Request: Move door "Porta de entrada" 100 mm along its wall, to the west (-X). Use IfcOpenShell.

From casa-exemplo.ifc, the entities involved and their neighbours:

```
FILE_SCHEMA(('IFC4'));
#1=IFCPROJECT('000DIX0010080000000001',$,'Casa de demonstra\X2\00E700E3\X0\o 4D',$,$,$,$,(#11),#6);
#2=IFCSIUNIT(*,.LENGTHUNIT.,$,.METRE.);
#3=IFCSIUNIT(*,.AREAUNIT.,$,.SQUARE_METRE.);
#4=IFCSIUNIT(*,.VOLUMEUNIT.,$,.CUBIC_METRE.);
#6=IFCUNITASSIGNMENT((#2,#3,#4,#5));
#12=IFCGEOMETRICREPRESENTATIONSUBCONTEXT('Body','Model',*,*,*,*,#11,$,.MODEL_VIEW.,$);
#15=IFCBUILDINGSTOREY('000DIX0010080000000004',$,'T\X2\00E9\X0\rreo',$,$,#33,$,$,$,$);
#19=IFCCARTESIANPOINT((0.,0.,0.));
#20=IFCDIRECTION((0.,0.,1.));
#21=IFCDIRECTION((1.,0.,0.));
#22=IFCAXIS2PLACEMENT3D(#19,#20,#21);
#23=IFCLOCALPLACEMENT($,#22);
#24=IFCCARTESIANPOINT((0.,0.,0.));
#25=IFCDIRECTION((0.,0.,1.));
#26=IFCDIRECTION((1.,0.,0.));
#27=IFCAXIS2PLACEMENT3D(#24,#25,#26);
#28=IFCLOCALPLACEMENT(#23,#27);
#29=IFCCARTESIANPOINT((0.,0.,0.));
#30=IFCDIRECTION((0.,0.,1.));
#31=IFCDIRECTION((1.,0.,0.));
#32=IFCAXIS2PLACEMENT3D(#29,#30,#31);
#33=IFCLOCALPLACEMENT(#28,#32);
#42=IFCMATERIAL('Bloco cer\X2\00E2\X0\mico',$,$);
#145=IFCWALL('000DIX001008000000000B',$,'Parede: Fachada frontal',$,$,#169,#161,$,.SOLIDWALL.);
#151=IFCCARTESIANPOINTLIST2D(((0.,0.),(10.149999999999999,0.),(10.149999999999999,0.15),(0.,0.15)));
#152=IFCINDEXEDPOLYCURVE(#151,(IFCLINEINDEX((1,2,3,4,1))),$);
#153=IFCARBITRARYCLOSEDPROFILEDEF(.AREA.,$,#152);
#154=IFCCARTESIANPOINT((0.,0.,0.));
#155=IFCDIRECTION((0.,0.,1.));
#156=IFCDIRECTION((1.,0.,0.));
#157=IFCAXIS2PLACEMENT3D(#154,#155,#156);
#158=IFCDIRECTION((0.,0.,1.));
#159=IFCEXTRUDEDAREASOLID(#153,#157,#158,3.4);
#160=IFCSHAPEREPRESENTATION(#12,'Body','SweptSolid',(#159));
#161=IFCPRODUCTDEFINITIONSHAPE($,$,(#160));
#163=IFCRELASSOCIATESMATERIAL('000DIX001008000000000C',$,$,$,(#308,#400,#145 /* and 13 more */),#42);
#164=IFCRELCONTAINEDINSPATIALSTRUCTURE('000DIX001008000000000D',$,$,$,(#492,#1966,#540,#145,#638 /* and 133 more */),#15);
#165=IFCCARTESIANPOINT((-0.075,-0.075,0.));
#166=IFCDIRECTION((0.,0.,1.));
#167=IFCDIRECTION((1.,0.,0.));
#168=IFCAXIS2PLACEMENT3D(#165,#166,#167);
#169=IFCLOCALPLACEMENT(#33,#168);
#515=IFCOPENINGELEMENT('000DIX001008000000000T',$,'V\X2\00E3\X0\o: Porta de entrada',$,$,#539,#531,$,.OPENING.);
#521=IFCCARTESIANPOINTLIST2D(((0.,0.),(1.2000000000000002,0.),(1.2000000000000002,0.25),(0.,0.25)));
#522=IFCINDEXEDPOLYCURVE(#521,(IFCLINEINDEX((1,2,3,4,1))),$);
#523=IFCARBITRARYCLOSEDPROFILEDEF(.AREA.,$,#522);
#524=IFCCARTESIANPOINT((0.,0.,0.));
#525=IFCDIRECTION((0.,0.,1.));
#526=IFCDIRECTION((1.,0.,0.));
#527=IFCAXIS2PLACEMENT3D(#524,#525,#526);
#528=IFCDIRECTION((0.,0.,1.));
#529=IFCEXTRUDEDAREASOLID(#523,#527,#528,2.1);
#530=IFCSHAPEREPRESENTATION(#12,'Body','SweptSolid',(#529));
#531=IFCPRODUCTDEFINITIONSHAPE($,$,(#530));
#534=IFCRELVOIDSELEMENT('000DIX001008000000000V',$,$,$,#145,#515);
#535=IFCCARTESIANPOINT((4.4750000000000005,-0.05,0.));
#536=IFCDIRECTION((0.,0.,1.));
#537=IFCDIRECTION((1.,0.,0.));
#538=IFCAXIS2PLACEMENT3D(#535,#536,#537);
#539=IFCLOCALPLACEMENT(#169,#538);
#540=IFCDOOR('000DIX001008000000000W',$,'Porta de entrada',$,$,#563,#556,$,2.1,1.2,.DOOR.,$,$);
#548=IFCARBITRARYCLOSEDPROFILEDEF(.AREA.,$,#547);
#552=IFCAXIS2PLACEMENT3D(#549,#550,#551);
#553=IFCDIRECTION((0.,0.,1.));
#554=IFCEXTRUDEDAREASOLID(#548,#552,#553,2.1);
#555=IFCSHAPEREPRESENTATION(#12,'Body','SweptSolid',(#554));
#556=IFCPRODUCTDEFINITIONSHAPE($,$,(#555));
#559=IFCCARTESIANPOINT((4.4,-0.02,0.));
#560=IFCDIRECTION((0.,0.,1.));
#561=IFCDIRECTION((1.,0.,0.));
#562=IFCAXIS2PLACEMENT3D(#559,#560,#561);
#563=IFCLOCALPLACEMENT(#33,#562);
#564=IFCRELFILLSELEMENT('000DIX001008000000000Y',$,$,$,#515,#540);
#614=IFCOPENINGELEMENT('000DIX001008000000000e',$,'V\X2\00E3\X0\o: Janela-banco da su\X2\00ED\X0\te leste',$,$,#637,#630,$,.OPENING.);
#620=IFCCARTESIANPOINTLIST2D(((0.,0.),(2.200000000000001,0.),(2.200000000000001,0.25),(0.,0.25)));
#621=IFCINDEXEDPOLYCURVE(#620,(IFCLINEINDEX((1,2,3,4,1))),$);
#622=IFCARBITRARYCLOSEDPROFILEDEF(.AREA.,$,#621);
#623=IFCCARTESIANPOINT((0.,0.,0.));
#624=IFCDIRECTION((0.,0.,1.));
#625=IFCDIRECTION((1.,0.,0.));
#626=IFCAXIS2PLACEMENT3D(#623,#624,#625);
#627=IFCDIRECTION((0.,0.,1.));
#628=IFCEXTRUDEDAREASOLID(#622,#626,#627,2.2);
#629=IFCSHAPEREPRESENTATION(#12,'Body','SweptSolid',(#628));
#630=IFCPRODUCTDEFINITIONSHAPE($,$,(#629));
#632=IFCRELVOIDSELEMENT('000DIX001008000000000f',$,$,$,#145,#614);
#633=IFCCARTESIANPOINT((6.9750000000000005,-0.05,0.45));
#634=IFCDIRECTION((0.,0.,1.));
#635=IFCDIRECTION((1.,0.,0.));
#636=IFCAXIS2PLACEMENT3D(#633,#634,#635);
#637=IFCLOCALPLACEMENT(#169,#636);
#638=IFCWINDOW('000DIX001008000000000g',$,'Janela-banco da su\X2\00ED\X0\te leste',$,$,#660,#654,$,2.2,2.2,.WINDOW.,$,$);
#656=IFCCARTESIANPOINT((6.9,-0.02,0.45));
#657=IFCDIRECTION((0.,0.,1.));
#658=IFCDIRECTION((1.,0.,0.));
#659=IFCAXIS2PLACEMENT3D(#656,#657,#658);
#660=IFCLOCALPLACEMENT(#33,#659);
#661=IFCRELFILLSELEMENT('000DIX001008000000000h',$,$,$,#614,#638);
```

```python
import ifcopenshell
import ifcopenshell.api.geometry
import ifcopenshell.util.placement

model = ifcopenshell.open("casa-exemplo.ifc")

door = model.by_id(540)
opening = door.FillsVoids[0].RelatingOpeningElement
wall = opening.VoidsElements[0].RelatingBuildingElement

wall_matrix = ifcopenshell.util.placement.get_local_placement(wall.ObjectPlacement)
shift = wall_matrix[:3, 0] * -0.1
before = ifcopenshell.util.placement.get_local_placement(door.ObjectPlacement)[:3, 3].copy()

# The door is not placed relative to its opening, so move both.
for product in (opening, door):
    matrix = ifcopenshell.util.placement.get_local_placement(product.ObjectPlacement)
    matrix[:3, 3] += shift
    ifcopenshell.api.geometry.edit_object_placement(model, product=product, matrix=matrix, is_si=False)

after = ifcopenshell.util.placement.get_local_placement(door.ObjectPlacement)[:3, 3]
print("door moved by", (after - before).round(3) + 0.0)

model.write("casa-exemplo_rev.ifc")
```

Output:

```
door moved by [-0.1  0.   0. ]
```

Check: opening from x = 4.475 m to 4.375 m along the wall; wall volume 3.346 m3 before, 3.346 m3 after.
